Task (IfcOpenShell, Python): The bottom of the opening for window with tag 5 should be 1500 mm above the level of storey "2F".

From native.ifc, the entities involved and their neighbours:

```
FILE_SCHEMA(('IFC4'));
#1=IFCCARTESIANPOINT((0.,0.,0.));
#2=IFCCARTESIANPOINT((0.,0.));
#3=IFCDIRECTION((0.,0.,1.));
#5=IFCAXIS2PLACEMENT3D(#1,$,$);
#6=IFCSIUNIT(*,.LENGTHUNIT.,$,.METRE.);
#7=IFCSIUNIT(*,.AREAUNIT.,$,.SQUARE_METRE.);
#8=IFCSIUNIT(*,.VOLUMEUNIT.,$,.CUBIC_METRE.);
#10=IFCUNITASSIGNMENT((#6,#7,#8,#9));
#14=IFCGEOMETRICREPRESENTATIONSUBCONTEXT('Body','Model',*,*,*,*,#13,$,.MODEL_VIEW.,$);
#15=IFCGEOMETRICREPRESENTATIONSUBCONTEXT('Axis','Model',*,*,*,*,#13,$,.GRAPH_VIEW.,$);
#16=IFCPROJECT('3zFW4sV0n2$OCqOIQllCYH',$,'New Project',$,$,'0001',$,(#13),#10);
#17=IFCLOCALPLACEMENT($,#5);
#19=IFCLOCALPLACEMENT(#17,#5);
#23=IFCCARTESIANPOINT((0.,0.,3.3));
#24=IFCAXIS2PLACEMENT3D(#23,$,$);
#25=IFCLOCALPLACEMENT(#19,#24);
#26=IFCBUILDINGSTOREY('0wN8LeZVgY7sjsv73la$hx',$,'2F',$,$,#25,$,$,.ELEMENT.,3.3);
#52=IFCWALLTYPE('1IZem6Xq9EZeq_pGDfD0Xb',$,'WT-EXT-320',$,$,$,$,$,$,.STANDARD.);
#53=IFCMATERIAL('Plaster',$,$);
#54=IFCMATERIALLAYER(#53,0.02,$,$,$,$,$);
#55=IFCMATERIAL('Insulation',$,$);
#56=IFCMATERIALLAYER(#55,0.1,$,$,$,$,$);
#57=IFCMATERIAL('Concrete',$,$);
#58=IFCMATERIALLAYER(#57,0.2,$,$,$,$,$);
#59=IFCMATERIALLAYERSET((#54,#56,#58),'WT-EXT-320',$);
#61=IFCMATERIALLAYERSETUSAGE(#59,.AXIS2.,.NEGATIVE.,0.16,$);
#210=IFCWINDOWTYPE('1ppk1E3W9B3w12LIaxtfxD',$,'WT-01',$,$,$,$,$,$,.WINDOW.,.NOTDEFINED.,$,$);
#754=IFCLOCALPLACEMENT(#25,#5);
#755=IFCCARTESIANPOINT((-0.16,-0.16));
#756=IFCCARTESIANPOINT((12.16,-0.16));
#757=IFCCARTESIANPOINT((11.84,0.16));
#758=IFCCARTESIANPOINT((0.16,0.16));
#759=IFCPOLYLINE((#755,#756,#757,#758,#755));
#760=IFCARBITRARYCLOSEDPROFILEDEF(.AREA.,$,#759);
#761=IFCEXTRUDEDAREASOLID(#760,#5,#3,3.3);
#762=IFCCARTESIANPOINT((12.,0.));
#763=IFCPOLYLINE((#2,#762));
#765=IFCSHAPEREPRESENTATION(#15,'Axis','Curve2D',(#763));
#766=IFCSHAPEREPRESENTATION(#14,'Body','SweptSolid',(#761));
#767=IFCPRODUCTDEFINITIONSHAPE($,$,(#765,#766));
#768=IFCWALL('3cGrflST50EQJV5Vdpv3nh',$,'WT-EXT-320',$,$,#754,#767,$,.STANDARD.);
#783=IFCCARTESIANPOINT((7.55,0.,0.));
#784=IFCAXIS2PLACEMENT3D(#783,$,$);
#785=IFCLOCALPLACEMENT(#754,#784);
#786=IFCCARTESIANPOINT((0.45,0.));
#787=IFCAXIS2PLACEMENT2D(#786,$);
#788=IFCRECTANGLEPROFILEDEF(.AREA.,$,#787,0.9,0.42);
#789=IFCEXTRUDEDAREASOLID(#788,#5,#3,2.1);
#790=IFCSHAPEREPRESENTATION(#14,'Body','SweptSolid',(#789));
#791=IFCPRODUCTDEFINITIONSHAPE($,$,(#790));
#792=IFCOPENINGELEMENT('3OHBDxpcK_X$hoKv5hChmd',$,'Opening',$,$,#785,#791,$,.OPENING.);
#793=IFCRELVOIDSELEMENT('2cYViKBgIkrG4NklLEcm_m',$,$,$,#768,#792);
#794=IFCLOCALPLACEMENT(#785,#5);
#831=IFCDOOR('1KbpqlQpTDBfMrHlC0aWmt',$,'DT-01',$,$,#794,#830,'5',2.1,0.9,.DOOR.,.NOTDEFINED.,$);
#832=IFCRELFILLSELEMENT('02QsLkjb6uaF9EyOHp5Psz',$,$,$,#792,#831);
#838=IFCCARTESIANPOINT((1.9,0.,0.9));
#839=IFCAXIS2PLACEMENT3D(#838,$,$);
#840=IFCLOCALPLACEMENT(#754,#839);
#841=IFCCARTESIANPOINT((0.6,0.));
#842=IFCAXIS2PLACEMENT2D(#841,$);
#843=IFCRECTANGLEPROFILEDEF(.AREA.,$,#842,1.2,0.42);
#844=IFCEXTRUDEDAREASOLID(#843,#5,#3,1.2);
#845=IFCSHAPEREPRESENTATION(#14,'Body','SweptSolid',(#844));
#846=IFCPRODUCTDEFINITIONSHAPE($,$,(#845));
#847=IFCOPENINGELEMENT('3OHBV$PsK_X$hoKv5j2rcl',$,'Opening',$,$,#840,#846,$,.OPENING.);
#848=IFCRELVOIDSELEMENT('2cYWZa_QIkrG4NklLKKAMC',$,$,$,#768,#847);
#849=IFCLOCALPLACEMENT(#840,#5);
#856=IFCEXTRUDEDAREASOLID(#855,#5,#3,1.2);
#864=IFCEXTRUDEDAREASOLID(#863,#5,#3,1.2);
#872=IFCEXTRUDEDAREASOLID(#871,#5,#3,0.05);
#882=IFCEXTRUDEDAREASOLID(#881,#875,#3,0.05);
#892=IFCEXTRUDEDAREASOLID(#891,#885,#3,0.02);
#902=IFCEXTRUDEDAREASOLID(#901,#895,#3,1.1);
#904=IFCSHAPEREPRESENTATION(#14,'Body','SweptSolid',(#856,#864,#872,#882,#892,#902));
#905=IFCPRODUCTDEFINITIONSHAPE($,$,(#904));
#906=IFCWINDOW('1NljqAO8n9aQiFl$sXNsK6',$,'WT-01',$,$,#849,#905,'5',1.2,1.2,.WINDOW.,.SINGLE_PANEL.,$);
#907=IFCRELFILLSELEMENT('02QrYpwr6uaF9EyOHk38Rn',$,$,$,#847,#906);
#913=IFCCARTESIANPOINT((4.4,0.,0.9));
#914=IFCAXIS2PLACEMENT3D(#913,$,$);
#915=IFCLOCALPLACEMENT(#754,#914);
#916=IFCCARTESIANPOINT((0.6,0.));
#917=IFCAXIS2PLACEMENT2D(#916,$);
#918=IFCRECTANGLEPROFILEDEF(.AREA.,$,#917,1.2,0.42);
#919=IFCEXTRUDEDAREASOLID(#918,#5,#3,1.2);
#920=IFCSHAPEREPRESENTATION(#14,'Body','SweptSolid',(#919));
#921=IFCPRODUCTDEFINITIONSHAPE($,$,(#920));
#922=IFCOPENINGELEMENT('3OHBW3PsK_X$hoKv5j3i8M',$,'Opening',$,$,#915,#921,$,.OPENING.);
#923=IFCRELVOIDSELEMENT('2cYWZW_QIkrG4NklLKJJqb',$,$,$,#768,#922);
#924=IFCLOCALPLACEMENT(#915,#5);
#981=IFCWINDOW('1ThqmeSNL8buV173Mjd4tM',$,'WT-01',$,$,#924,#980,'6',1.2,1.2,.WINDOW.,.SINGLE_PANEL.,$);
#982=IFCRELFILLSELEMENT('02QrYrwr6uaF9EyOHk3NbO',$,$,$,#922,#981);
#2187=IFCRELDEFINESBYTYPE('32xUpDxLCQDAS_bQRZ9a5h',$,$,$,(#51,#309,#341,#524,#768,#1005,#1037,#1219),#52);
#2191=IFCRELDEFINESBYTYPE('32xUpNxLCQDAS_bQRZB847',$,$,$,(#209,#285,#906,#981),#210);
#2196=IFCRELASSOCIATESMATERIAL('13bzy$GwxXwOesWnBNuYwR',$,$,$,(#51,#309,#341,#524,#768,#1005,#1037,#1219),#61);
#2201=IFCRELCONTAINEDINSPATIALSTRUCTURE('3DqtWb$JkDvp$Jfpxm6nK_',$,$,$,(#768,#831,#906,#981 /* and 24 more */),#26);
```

```python
import numpy as np
import ifcopenshell
import ifcopenshell.api.geometry
import ifcopenshell.geom
import ifcopenshell.util.element
import ifcopenshell.util.placement
import ifcopenshell.util.shape
import ifcopenshell.util.unit

model = ifcopenshell.open("native.ifc")
unit_scale = ifcopenshell.util.unit.calculate_unit_scale(model)

window = model.by_guid("1NljqAO8n9aQiFl$sXNsK6")
opening = window.FillsVoids[0].RelatingOpeningElement
storey = ifcopenshell.util.element.get_container(window, ifc_class="IfcBuildingStorey")
level = ifcopenshell.util.placement.get_local_placement(storey.ObjectPlacement)[2, 3]

# The opening's origin need not be at the sill, so measure its lowest point.
shape = ifcopenshell.geom.create_shape(ifcopenshell.geom.settings(), opening)
bottom = ifcopenshell.util.shape.get_shape_bottom_elevation(shape, shape.geometry) / unit_scale
dz = level + 1.5 / unit_scale - bottom

shift = np.array([0.0, 0.0, dz])
# The window is placed relative to its opening, so it follows when the opening moves.
matrix = ifcopenshell.util.placement.get_local_placement(opening.ObjectPlacement)
matrix[:3, 3] += shift
ifcopenshell.api.geometry.edit_object_placement(
    model, product=opening, matrix=matrix, is_si=False, should_transform_children=True
)

print(f"moved by {dz * unit_scale:+.3f} m")

model.write("native-out.ifc")
```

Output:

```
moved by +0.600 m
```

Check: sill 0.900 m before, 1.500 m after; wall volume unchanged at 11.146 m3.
